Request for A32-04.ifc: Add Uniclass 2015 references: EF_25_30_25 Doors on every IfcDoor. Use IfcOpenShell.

First a look at what the model holds.

```python
import ifcopenshell

model = ifcopenshell.open("A32-04.ifc")
print(model.schema)
print("classifications:", [c.Name for c in model.by_type("IfcClassification")])
for ifc_class in ("IfcDoor", "IfcRoof", "IfcStair", "IfcWall", "IfcWindow"):
    print(ifc_class, len(model.by_type(ifc_class)))
```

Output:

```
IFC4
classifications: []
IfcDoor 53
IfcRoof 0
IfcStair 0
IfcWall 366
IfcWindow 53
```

```python
import ifcopenshell
import ifcopenshell.api.classification

model = ifcopenshell.open("A32-04.ifc")

system = ifcopenshell.api.classification.add_classification(model, classification="Uniclass 2015")

codes = {
    "IfcDoor": ("EF_25_30_25", "Doors"),
}
for ifc_class, (code, name) in codes.items():
    products = model.by_type(ifc_class)
    ifcopenshell.api.classification.add_reference(
        model, products=products, classification=system, identification=code, name=name
    )
    print(code, len(products))

model.write("A32-04_edited.ifc")
```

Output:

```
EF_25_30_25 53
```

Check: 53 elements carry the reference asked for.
